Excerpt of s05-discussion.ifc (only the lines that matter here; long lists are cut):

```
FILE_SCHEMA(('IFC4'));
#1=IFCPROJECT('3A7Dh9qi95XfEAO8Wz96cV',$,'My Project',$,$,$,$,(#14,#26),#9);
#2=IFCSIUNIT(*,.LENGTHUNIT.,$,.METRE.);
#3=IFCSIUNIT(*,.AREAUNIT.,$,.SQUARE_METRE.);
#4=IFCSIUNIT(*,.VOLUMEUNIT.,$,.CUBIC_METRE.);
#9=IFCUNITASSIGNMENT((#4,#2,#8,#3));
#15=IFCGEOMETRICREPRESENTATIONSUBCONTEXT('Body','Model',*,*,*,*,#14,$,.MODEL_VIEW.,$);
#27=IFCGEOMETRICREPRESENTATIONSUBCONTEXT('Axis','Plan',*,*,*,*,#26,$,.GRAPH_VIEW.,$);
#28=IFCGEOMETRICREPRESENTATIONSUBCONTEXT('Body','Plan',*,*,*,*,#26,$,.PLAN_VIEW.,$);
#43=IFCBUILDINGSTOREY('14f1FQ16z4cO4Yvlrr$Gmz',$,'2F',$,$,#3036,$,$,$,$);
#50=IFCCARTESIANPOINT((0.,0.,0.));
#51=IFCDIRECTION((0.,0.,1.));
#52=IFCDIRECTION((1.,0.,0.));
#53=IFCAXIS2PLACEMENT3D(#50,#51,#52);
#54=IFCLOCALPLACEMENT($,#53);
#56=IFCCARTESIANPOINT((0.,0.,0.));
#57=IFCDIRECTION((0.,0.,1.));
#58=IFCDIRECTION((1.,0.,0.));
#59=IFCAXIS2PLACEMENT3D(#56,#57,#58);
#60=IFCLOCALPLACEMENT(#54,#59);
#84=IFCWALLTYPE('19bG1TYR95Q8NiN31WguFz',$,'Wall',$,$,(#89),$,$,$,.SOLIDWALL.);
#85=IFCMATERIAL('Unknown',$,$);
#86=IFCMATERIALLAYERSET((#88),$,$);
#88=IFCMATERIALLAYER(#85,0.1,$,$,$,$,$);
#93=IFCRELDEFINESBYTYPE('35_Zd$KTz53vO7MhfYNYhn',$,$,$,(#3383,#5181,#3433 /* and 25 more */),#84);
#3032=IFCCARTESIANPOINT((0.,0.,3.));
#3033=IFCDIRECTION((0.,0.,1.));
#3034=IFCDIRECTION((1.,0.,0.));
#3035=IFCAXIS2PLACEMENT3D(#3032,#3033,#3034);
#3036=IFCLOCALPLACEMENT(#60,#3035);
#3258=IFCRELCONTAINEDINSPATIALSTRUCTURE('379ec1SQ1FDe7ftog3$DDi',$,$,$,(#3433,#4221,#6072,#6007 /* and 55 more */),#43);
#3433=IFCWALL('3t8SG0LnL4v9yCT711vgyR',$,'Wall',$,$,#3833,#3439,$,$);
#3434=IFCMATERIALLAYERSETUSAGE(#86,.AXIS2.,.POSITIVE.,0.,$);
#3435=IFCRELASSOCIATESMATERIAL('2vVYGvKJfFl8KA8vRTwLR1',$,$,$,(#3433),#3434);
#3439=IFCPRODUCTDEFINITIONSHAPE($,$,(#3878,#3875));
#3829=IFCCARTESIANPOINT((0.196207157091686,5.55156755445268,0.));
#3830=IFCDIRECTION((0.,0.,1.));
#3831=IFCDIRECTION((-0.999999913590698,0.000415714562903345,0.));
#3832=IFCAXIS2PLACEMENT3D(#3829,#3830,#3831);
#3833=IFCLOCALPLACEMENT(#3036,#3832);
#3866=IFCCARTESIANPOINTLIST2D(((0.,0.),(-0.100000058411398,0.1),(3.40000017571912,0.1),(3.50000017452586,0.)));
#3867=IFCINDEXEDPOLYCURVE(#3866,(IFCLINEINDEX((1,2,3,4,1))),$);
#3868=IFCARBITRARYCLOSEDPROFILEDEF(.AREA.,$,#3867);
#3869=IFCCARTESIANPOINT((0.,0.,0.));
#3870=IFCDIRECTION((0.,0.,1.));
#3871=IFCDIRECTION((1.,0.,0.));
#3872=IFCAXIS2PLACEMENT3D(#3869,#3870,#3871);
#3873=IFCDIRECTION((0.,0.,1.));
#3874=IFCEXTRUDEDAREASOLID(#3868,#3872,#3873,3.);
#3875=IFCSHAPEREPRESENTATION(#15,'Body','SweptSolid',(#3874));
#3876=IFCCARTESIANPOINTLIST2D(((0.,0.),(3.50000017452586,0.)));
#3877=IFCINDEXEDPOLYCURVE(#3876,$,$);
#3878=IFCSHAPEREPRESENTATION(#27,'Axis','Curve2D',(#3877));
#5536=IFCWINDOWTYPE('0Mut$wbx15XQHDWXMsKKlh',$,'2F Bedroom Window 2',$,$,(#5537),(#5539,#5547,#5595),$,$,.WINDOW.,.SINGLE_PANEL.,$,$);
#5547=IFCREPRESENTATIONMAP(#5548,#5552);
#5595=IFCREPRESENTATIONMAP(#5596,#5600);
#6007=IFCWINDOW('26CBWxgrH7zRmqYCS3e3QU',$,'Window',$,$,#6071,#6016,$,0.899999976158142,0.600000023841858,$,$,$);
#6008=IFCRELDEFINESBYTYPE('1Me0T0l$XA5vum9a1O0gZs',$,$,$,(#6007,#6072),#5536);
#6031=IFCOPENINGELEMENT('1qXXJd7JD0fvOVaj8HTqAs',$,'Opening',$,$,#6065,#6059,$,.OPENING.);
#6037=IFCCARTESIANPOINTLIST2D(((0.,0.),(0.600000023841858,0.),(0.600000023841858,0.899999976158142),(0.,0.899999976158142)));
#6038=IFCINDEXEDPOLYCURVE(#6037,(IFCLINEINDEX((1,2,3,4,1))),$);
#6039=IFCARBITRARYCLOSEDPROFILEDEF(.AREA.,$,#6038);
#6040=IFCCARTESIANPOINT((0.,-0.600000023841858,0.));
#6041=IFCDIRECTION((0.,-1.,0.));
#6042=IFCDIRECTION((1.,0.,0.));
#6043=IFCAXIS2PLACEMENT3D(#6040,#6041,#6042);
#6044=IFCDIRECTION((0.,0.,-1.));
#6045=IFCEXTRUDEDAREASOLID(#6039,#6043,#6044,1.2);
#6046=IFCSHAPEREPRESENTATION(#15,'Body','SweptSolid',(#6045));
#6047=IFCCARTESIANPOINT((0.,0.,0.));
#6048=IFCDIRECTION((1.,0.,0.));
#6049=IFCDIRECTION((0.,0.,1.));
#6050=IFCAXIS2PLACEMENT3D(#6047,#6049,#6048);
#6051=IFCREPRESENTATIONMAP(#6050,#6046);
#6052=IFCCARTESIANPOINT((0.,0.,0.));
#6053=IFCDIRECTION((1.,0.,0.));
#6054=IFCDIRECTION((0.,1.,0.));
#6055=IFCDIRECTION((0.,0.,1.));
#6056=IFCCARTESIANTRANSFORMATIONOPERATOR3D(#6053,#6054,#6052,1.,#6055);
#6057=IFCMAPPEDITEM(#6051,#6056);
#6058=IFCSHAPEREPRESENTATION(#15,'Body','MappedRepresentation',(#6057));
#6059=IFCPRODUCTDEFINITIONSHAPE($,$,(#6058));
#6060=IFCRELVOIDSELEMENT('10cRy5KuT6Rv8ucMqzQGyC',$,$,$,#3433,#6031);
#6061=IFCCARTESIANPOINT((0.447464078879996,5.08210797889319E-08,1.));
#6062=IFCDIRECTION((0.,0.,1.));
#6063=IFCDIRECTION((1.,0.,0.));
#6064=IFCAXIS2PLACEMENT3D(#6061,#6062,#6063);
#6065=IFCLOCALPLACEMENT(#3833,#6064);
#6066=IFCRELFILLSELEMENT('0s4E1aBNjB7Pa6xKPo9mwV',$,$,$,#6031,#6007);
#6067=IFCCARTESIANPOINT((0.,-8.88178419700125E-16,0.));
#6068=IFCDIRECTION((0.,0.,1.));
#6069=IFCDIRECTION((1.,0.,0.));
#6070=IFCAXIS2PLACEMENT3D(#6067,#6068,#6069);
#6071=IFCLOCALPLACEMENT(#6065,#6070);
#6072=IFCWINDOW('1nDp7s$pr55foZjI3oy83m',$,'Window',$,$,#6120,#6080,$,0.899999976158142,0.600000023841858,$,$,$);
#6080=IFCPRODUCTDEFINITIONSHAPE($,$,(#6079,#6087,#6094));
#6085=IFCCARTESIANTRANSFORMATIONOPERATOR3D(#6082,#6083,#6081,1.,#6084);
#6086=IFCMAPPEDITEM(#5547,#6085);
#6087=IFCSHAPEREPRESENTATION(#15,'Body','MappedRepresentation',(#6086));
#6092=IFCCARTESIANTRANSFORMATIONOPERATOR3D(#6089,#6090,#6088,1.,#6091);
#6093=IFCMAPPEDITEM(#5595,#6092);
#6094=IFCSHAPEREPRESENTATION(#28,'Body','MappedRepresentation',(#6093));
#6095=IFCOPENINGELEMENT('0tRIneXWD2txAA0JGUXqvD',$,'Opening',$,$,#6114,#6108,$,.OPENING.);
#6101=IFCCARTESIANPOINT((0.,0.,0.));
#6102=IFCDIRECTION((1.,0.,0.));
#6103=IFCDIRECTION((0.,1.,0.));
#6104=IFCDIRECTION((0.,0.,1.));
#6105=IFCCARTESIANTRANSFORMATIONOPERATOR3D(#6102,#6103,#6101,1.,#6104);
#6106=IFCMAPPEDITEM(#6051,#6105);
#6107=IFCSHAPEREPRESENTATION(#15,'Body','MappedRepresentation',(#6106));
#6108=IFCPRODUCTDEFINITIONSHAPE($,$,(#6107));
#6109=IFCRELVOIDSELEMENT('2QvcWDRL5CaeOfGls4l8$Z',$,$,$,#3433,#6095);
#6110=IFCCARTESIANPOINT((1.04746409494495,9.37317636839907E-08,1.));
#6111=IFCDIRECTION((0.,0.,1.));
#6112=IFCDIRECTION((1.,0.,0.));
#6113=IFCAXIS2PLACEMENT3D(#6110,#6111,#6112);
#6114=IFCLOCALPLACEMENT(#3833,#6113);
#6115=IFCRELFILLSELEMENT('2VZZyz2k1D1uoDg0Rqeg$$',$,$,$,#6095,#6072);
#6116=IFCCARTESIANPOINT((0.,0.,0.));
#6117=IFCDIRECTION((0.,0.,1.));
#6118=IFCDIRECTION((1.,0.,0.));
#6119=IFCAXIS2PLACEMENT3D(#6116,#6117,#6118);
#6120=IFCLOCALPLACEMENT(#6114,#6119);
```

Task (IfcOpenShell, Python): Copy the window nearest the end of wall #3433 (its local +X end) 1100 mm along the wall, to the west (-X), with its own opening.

```python
import ifcopenshell
import ifcopenshell.api.feature
import ifcopenshell.api.geometry
import ifcopenshell.api.root
import ifcopenshell.geom
import ifcopenshell.util.element
import ifcopenshell.util.placement
import ifcopenshell.util.shape
import ifcopenshell.util.unit

model = ifcopenshell.open("s05-discussion.ifc")
unit_scale = ifcopenshell.util.unit.calculate_unit_scale(model)
settings = ifcopenshell.geom.settings()


def volume(element):
    """Net volume in cubic metres, openings subtracted."""
    shape = ifcopenshell.geom.create_shape(settings, element)
    return ifcopenshell.util.shape.get_volume(shape.geometry)


window = model.by_guid("1nDp7s$pr55foZjI3oy83m")
opening = window.FillsVoids[0].RelatingOpeningElement
wall = opening.VoidsElements[0].RelatingBuildingElement
before = volume(wall)
shift = ifcopenshell.util.placement.get_local_placement(wall.ObjectPlacement)[:3, 0] * 1.1 / unit_scale

# copy_class copies the void relationship, type, container and properties, but no geometry.
new_opening = ifcopenshell.api.root.copy_class(model, product=opening)
new_opening.Representation = ifcopenshell.util.element.copy_deep(
    model, opening.Representation, exclude=["IfcGeometricRepresentationContext", "IfcRepresentationMap"]
)
new_window = ifcopenshell.api.root.copy_class(model, product=window)
new_window.Representation = ifcopenshell.util.element.copy_deep(
    model, window.Representation, exclude=["IfcGeometricRepresentationContext", "IfcRepresentationMap"]
)
ifcopenshell.api.feature.add_filling(model, opening=new_opening, element=new_window)

for old, new in ((opening, new_opening), (window, new_window)):
    matrix = ifcopenshell.util.placement.get_local_placement(old.ObjectPlacement)
    matrix[:3, 3] += shift
    ifcopenshell.api.geometry.edit_object_placement(model, product=new, matrix=matrix, is_si=False)

after = volume(wall)

print(f"wall volume {before:.3f} -> {after:.3f} m3")

model.write("s05-discussion_edited.ifc")
```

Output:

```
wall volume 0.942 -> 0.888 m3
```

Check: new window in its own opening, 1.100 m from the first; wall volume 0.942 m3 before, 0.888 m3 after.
